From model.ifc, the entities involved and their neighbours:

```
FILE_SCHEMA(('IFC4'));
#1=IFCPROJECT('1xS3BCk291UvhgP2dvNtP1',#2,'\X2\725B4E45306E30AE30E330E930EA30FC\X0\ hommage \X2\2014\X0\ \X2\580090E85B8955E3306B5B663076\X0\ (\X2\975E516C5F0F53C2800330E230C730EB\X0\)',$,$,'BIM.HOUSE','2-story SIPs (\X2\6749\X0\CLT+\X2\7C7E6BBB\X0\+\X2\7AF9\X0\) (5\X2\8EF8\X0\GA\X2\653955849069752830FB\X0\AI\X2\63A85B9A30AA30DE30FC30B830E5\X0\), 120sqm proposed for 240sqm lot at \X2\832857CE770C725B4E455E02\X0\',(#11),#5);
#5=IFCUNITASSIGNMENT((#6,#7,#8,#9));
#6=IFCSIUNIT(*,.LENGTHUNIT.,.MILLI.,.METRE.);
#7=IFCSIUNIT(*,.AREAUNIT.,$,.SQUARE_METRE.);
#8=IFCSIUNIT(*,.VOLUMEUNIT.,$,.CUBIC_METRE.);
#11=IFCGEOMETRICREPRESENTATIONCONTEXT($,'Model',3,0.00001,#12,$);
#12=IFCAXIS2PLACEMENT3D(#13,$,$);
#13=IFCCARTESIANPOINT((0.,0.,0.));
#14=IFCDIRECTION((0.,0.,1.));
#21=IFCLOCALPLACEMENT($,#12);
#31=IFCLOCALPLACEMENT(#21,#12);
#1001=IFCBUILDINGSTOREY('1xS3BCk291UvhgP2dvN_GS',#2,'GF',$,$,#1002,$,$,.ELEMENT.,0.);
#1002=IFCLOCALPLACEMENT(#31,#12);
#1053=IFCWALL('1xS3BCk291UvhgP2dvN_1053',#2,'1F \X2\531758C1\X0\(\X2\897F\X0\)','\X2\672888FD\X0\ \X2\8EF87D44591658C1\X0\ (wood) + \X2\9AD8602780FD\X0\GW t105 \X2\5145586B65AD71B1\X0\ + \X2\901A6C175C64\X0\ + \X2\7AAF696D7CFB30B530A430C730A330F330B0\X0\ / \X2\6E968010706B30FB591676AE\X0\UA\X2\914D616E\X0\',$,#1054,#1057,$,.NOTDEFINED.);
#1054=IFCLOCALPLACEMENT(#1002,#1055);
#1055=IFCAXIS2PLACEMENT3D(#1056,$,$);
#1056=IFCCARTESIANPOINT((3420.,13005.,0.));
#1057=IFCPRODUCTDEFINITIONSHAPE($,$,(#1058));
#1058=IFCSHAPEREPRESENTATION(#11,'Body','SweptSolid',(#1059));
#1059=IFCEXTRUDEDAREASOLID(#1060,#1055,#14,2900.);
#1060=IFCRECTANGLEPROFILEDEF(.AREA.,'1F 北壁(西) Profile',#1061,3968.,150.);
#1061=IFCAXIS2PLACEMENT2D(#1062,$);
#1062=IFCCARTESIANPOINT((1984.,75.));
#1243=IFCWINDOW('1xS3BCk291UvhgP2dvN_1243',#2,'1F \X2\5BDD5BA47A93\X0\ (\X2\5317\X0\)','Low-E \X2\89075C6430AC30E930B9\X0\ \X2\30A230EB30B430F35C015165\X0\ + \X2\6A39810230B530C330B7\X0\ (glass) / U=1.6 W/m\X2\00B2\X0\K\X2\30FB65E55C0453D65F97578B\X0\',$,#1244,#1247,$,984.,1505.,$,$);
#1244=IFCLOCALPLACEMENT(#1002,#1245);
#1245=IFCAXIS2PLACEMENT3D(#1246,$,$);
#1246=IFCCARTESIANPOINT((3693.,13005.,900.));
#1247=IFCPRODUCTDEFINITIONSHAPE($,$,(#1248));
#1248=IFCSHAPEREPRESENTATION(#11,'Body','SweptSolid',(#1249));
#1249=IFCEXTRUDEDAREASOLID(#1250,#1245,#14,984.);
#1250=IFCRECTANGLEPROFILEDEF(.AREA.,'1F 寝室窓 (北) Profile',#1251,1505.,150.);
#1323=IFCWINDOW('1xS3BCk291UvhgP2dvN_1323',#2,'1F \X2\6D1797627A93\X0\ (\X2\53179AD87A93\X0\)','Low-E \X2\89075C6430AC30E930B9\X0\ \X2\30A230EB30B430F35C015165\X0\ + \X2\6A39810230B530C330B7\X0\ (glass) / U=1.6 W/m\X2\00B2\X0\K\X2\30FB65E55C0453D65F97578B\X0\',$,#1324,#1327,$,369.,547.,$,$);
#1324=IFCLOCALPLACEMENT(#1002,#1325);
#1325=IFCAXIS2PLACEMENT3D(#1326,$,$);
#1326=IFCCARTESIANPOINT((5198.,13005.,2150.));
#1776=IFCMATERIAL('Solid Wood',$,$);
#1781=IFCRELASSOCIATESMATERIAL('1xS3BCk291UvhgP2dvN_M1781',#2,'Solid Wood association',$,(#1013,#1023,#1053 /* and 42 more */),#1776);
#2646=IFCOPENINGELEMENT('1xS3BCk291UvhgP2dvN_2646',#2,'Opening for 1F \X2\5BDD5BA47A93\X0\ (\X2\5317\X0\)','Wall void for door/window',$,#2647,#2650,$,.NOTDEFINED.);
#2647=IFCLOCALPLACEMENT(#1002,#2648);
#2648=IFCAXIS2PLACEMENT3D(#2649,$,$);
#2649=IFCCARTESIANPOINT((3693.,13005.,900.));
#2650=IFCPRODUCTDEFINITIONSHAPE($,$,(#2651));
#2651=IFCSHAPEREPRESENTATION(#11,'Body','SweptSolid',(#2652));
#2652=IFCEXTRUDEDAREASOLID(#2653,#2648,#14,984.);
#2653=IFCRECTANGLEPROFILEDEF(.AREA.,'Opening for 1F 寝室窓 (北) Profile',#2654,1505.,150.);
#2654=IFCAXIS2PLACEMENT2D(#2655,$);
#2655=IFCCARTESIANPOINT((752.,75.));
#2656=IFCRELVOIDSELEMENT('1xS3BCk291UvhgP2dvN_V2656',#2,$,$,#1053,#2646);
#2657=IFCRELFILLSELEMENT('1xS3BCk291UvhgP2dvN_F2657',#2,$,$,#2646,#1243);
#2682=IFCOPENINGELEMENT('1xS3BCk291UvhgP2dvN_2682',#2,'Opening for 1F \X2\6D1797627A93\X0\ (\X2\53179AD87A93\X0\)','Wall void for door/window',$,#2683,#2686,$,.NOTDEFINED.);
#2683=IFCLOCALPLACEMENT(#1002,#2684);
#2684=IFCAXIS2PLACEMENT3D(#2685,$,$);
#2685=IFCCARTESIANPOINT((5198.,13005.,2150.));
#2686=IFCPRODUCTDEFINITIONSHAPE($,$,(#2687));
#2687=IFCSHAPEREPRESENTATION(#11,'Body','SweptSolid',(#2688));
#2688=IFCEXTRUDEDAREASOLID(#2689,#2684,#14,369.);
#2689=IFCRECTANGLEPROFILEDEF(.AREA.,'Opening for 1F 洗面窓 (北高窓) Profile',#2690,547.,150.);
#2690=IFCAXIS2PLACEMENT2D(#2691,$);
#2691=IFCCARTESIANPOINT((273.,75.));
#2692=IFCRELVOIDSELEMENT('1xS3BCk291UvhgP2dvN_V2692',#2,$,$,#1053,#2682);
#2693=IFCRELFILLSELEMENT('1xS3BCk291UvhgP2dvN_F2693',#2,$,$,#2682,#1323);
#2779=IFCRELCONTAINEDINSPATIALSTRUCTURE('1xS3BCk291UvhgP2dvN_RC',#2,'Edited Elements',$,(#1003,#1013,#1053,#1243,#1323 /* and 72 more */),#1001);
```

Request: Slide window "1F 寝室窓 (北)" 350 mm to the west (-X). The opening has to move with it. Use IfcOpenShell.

```python
import ifcopenshell
import ifcopenshell.api.geometry
import ifcopenshell.util.placement
import ifcopenshell.util.unit

model = ifcopenshell.open("model.ifc")
unit_scale = ifcopenshell.util.unit.calculate_unit_scale(model)

window = model.by_guid("1xS3BCk291UvhgP2dvN_1243")
opening = window.FillsVoids[0].RelatingOpeningElement
wall = opening.VoidsElements[0].RelatingBuildingElement

wall_matrix = ifcopenshell.util.placement.get_local_placement(wall.ObjectPlacement)
shift = wall_matrix[:3, 0] * -0.35 / unit_scale
before = ifcopenshell.util.placement.get_local_placement(window.ObjectPlacement)[:3, 3].copy()

# The window is not placed relative to its opening, so move both.
for product in (opening, window):
    matrix = ifcopenshell.util.placement.get_local_placement(product.ObjectPlacement)
    matrix[:3, 3] += shift
    ifcopenshell.api.geometry.edit_object_placement(model, product=product, matrix=matrix, is_si=False)

after = ifcopenshell.util.placement.get_local_placement(window.ObjectPlacement)[:3, 3]
print("window moved by", (after - before).round(3) + 0.0)

model.write("model_updated.ifc")
```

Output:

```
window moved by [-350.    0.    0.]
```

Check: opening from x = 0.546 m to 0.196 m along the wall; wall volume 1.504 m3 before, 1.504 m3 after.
